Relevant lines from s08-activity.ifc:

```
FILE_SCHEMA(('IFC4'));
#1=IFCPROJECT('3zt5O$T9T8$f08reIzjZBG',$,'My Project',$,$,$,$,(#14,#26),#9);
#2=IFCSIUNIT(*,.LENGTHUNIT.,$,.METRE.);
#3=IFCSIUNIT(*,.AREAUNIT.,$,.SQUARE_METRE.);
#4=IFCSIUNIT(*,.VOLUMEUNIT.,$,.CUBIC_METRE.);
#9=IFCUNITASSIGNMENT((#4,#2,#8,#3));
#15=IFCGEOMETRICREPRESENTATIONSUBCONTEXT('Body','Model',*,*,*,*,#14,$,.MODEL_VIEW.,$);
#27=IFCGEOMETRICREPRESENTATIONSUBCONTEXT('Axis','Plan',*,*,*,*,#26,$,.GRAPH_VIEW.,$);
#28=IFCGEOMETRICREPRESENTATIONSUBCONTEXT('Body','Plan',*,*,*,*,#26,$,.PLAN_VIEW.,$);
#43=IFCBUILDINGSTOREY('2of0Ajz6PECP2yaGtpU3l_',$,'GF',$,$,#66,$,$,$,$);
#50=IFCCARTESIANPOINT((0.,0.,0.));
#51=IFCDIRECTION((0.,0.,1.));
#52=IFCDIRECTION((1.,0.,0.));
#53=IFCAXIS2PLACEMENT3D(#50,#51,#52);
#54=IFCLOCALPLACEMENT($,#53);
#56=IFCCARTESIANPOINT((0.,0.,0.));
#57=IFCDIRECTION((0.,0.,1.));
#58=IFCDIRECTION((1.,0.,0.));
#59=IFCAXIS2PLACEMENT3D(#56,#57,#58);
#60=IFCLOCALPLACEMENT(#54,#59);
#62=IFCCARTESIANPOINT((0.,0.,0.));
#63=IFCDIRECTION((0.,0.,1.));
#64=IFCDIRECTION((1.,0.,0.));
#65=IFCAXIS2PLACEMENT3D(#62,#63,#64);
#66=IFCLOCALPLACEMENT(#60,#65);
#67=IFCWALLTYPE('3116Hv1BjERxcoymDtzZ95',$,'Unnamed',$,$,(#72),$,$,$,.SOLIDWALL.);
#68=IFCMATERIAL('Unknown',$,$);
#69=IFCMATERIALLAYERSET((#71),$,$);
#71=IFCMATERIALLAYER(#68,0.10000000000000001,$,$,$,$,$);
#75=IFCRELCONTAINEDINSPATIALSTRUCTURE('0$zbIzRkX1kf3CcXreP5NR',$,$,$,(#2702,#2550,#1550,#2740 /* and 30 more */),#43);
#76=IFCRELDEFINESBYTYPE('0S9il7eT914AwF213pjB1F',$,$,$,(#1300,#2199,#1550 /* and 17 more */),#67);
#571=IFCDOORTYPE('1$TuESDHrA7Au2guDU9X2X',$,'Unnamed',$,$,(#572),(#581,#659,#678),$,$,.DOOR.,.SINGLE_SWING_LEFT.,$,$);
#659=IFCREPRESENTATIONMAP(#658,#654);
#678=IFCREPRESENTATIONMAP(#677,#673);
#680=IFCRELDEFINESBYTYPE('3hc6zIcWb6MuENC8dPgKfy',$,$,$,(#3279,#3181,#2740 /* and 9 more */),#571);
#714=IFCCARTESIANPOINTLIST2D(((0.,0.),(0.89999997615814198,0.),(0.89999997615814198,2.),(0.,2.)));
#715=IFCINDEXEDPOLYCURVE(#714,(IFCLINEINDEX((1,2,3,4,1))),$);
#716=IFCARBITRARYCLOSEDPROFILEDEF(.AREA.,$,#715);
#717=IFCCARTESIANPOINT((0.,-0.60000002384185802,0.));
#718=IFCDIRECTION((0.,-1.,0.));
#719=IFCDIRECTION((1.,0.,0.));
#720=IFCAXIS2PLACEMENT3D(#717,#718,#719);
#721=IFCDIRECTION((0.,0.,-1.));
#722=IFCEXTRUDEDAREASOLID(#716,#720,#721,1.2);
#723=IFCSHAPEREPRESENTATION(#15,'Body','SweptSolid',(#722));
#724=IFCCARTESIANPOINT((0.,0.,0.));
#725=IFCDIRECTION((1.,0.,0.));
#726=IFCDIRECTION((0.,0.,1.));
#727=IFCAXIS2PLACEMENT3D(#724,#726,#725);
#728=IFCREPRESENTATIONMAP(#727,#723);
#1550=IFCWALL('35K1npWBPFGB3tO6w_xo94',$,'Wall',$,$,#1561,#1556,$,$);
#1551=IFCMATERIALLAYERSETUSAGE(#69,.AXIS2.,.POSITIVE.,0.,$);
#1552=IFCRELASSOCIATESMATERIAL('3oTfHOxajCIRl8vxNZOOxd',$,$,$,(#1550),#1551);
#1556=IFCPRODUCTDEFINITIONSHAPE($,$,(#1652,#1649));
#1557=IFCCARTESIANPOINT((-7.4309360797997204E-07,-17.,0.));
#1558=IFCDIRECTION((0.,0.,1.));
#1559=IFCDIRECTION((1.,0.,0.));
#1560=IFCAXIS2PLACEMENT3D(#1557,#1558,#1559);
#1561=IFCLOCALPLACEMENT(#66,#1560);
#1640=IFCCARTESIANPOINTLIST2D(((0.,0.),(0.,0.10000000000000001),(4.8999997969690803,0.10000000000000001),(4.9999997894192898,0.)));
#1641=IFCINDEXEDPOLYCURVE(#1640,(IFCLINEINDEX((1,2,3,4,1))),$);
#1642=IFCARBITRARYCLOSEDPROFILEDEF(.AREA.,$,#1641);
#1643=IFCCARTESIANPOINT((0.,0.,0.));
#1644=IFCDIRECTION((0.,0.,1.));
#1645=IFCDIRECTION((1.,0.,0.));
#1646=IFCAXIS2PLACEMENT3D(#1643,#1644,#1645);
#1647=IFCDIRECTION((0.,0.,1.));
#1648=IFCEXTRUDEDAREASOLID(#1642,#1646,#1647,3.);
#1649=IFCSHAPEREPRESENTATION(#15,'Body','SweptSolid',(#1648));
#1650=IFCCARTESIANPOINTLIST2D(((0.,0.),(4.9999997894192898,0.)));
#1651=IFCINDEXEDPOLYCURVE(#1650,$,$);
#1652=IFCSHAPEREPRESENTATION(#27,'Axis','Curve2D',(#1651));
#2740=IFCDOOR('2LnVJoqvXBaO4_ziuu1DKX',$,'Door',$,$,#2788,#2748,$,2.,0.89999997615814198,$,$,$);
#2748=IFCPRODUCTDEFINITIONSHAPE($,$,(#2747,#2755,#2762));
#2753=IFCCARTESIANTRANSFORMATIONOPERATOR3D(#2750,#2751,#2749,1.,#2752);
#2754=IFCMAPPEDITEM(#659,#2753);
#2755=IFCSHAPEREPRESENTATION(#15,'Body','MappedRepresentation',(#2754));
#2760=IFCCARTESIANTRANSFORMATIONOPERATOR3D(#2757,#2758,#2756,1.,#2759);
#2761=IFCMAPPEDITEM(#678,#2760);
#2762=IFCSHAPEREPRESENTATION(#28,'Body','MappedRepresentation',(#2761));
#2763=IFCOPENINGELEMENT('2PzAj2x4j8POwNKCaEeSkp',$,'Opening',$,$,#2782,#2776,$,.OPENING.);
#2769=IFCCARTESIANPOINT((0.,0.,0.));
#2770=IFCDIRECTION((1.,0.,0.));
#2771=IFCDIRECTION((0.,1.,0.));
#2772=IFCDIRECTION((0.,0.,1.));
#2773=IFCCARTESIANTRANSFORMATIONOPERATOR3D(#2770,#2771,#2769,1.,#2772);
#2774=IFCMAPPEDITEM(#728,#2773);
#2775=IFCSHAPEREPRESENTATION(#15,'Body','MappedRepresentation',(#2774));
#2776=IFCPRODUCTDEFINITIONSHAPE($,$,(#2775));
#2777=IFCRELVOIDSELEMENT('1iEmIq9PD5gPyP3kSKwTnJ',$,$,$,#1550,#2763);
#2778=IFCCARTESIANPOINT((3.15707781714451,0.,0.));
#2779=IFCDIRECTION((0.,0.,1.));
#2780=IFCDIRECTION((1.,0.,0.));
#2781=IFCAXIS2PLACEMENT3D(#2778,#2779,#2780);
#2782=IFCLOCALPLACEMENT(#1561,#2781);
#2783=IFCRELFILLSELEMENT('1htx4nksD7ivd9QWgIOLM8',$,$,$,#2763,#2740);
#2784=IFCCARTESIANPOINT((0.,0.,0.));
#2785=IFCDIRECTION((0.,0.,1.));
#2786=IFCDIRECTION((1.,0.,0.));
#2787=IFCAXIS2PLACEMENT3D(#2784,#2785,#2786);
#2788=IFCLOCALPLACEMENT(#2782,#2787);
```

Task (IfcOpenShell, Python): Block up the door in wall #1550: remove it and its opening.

```python
import ifcopenshell
import ifcopenshell.api.feature
import ifcopenshell.api.root
import ifcopenshell.geom
import ifcopenshell.util.shape

model = ifcopenshell.open("s08-activity.ifc")
settings = ifcopenshell.geom.settings()


def volume(element):
    """Net volume in cubic metres, openings subtracted."""
    shape = ifcopenshell.geom.create_shape(settings, element)
    return ifcopenshell.util.shape.get_volume(shape.geometry)


door = model.by_id(2740)
opening = door.FillsVoids[0].RelatingOpeningElement
wall = opening.VoidsElements[0].RelatingBuildingElement
before = volume(wall)

ifcopenshell.api.root.remove_product(model, product=door)
ifcopenshell.api.feature.remove_feature(model, feature=opening)

after = volume(wall)

print(f"wall volume {before:.3f} -> {after:.3f} m3")

model.write("s08-activity_v2.ifc")
```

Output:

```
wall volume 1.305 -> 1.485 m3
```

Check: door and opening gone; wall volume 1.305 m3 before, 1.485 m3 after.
